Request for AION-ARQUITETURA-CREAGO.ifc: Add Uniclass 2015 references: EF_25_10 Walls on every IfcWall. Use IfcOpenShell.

First a look at what the model holds.

```python
import ifcopenshell

model = ifcopenshell.open("AION-ARQUITETURA-CREAGO.ifc")
print(model.schema)
print("classifications:", [c.Name for c in model.by_type("IfcClassification")])
for ifc_class in ("IfcDoor", "IfcRoof", "IfcStair", "IfcWall", "IfcWindow"):
    print(ifc_class, len(model.by_type(ifc_class)))
```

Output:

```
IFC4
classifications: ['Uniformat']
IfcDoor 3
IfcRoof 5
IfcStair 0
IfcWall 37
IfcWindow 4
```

```python
import ifcopenshell
import ifcopenshell.api.classification

model = ifcopenshell.open("AION-ARQUITETURA-CREAGO.ifc")

system = ifcopenshell.api.classification.add_classification(model, classification="Uniclass 2015")

codes = {
    "IfcWall": ("EF_25_10", "Walls"),
}
for ifc_class, (code, name) in codes.items():
    products = model.by_type(ifc_class)
    ifcopenshell.api.classification.add_reference(
        model, products=products, classification=system, identification=code, name=name
    )
    print(code, len(products))

model.write("AION-ARQUITETURA-CREAGO_updated.ifc")
```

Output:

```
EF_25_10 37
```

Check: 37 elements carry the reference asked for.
